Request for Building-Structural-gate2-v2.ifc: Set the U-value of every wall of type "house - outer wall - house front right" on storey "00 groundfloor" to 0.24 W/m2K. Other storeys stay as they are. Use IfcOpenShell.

First a look at what the model holds.

```python
import ifcopenshell
import ifcopenshell.util.element

model = ifcopenshell.open("Building-Structural-gate2-v2.ifc")
print(model.schema)
storey = next(s for s in model.by_type("IfcBuildingStorey") if s.Name == "00 groundfloor")
walls = [e for e in ifcopenshell.util.element.get_decomposition(storey) if e.is_a("IfcWall")]
seen = {}
for e in walls:
    element_type = ifcopenshell.util.element.get_type(e)
    key = (element_type.Name if element_type != e and element_type else None, ifcopenshell.util.element.get_pset(e, "Pset_WallCommon", "ThermalTransmittance"))
    seen[key] = seen.get(key, 0) + 1
for (name, value), count in sorted(seen.items(), key=str):
    print(count, "x", name, "|", value)
```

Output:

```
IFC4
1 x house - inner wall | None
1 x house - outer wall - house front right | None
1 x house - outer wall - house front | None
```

```python
import ifcopenshell
import ifcopenshell.api.pset
import ifcopenshell.util.element

model = ifcopenshell.open("Building-Structural-gate2-v2.ifc")

storey = next(s for s in model.by_type("IfcBuildingStorey") if s.Name == "00 groundfloor")
walls = [e for e in ifcopenshell.util.element.get_decomposition(storey) if e.is_a("IfcWall")]

count = 0
for e in walls:
    element_type = ifcopenshell.util.element.get_type(e)
    if element_type in (None, e) or element_type.Name != "house - outer wall - house front right":
        continue
    # add_pset returns the element's existing set when there is one.
    pset = ifcopenshell.api.pset.add_pset(model, product=e, name="Pset_WallCommon")
    ifcopenshell.api.pset.edit_pset(model, pset=pset, properties={"ThermalTransmittance": 0.24})
    count += 1

print(count, "walls updated")

model.write("Building-Structural-gate2-v2_updated.ifc")
```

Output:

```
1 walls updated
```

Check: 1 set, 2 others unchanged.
